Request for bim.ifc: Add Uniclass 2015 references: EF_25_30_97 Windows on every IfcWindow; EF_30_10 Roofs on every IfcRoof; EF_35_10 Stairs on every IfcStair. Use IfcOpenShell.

First a look at what the model holds.

```python
import ifcopenshell

model = ifcopenshell.open("bim.ifc")
print(model.schema)
print("classifications:", [c.Name for c in model.by_type("IfcClassification")])
for ifc_class in ("IfcDoor", "IfcRoof", "IfcStair", "IfcWall", "IfcWindow"):
    print(ifc_class, len(model.by_type(ifc_class)))
```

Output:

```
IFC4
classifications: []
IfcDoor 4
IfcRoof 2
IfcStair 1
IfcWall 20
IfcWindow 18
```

```python
import ifcopenshell
import ifcopenshell.api.classification

model = ifcopenshell.open("bim.ifc")

system = ifcopenshell.api.classification.add_classification(model, classification="Uniclass 2015")

codes = {
    "IfcWindow": ("EF_25_30_97", "Windows"),
    "IfcRoof": ("EF_30_10", "Roofs"),
    "IfcStair": ("EF_35_10", "Stairs"),
}
for ifc_class, (code, name) in codes.items():
    products = model.by_type(ifc_class)
    ifcopenshell.api.classification.add_reference(
        model, products=products, classification=system, identification=code, name=name
    )
    print(code, len(products))

model.write("bim_rev.ifc")
```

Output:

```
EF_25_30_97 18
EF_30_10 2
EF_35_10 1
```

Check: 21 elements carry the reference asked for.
